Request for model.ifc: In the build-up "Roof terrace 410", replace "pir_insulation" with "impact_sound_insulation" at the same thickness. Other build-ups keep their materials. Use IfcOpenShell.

First a look at what the model holds.

```python
import ifcopenshell
import ifcopenshell.util.element

model = ifcopenshell.open("model.ifc")
print(model.schema)
for layer_set in model.by_type("IfcMaterialLayerSet"):
    if layer_set.LayerSetName == "Roof terrace 410":
        for layer in layer_set.MaterialLayers:
            print(layer.id(), layer.Material and layer.Material.Name, layer.LayerThickness, sep=" | ")
        print(len(ifcopenshell.util.element.get_elements_by_material(model, layer_set)), "elements and types use it")
print(sorted(m.Name for m in model.by_type("IfcMaterial") if m.Name)[:60])
```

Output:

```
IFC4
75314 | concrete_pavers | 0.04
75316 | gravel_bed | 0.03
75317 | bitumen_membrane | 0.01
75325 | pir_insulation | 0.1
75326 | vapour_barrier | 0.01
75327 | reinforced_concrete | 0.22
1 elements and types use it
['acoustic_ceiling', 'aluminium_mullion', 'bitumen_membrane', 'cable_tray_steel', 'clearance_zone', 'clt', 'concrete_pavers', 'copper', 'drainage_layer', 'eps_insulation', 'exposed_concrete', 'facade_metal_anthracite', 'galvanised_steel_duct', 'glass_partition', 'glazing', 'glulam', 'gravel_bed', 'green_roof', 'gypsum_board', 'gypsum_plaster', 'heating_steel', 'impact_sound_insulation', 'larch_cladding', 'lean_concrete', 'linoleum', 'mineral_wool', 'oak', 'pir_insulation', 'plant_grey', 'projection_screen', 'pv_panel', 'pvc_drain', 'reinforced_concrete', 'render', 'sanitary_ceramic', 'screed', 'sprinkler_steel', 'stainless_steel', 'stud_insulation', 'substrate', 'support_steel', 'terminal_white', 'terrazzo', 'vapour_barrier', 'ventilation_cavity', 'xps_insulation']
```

```python
import ifcopenshell
import ifcopenshell.api.material

model = ifcopenshell.open("model.ifc")

layer_set = next(s for s in model.by_type("IfcMaterialLayerSet") if s.LayerSetName == "Roof terrace 410")
layer = next(l for l in layer_set.MaterialLayers if l.Material and l.Material.Name == "pir_insulation")
material = next(m for m in model.by_type("IfcMaterial") if m.Name == "impact_sound_insulation")

# Point this one layer at the other material; renaming the old one would change it everywhere.
ifcopenshell.api.material.edit_layer(model, layer=layer, attributes={"Name": material.Name}, material=material)

print([l.Material.Name if l.Material else None for l in layer_set.MaterialLayers])

model.write("model_rev.ifc")
```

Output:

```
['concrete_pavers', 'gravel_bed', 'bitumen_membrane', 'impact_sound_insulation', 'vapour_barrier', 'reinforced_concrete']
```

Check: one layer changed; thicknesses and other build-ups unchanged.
